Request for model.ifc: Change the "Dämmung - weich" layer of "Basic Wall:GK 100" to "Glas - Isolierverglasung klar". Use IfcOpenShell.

First a look at what the model holds.

```python
import ifcopenshell
import ifcopenshell.util.element

model = ifcopenshell.open("model.ifc")
print(model.schema)
for layer_set in model.by_type("IfcMaterialLayerSet"):
    if layer_set.LayerSetName == "Basic Wall:GK 100":
        for layer in layer_set.MaterialLayers:
            print(layer.id(), layer.Material and layer.Material.Name, layer.LayerThickness, sep=" | ")
        print(len(ifcopenshell.util.element.get_elements_by_material(model, layer_set)), "elements and types use it")
print(sorted(m.Name for m in model.by_type("IfcMaterial") if m.Name)[:60])
```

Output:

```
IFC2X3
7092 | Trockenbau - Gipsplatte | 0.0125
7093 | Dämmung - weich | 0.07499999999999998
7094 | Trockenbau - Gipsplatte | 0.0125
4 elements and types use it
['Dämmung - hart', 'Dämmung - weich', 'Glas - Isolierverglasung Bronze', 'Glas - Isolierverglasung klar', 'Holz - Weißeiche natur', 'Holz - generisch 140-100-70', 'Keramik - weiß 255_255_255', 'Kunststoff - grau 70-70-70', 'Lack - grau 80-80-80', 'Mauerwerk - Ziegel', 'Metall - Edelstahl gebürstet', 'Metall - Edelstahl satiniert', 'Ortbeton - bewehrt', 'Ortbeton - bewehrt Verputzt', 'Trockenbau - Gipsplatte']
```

```python
import ifcopenshell
import ifcopenshell.api.material

model = ifcopenshell.open("model.ifc")

layer_set = next(s for s in model.by_type("IfcMaterialLayerSet") if s.LayerSetName == "Basic Wall:GK 100")
layer = next(l for l in layer_set.MaterialLayers if l.Material and l.Material.Name == "Dämmung - weich")
material = next(m for m in model.by_type("IfcMaterial") if m.Name == "Glas - Isolierverglasung klar")

# Point this one layer at the other material; renaming the old one would change it everywhere.
ifcopenshell.api.material.edit_layer(model, layer=layer, attributes={}, material=material)

print([l.Material.Name if l.Material else None for l in layer_set.MaterialLayers])

model.write("model_updated.ifc")
```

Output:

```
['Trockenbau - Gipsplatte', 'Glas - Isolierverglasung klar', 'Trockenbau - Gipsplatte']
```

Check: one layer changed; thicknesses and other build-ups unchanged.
